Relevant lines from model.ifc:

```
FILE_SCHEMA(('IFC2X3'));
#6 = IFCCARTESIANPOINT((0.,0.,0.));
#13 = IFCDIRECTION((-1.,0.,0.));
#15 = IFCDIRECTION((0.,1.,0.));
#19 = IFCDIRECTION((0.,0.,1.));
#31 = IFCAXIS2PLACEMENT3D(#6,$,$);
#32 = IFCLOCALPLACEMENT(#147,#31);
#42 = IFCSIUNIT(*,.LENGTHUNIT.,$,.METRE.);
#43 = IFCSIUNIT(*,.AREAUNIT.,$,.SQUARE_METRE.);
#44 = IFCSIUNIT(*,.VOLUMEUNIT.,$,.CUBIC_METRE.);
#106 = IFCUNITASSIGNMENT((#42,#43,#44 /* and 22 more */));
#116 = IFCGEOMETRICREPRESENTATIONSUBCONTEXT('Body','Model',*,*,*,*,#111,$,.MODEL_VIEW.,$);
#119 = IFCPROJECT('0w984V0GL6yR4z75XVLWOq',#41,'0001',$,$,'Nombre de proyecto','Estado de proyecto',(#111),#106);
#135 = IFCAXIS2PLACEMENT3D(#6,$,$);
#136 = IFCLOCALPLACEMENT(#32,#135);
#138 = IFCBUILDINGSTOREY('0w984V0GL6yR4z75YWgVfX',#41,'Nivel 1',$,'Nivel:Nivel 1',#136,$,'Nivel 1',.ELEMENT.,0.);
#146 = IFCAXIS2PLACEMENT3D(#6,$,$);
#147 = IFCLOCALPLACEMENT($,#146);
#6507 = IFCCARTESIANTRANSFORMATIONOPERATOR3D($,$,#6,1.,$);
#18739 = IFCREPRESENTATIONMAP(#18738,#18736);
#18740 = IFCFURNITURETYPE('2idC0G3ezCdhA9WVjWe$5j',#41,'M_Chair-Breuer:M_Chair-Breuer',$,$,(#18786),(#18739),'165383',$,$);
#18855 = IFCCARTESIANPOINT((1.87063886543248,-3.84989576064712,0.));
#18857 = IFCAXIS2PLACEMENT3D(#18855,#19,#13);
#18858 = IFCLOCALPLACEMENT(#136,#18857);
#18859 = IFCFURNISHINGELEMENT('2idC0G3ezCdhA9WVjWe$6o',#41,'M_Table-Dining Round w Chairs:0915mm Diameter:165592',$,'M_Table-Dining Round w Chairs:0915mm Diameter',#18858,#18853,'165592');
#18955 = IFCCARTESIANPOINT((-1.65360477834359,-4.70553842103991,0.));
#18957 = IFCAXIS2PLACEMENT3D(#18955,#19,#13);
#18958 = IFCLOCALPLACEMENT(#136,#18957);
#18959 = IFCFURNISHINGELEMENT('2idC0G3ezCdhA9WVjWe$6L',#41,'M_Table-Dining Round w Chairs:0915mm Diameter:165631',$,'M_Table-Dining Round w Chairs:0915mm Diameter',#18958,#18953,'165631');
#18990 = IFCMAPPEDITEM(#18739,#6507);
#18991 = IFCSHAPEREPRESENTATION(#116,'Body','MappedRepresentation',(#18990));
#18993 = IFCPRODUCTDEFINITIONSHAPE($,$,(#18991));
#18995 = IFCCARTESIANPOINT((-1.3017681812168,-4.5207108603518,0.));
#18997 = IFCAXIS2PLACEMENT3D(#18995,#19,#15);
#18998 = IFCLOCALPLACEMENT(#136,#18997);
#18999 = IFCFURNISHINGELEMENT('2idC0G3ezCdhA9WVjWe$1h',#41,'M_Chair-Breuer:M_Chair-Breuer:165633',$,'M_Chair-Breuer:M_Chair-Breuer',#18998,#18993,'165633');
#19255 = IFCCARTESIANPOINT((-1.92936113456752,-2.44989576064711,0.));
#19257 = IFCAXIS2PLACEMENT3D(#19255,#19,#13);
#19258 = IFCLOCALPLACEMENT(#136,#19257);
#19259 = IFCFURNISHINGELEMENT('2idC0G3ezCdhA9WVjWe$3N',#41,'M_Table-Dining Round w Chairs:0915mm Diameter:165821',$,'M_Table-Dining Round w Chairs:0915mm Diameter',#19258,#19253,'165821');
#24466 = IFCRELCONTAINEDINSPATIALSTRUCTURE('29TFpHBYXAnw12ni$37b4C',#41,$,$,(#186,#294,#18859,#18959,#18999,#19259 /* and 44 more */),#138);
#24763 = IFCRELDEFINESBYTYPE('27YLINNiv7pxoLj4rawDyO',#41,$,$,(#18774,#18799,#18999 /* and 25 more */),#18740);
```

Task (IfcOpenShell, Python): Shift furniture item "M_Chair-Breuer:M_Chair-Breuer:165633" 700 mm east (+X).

```python
import ifcopenshell
import ifcopenshell.api.geometry
import ifcopenshell.util.placement
import ifcopenshell.util.unit

model = ifcopenshell.open("model.ifc")
unit_scale = ifcopenshell.util.unit.calculate_unit_scale(model)

item = model.by_guid("2idC0G3ezCdhA9WVjWe$1h")
matrix = ifcopenshell.util.placement.get_local_placement(item.ObjectPlacement)
matrix[0, 3] += 0.7 / unit_scale
ifcopenshell.api.geometry.edit_object_placement(model, product=item, matrix=matrix, is_si=False)

print(ifcopenshell.util.placement.get_local_placement(item.ObjectPlacement).round(3) + 0.0)

model.write("model_v2.ifc")
```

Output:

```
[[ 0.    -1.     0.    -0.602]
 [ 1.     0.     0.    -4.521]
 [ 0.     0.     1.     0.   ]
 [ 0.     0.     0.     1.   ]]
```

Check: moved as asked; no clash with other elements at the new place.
